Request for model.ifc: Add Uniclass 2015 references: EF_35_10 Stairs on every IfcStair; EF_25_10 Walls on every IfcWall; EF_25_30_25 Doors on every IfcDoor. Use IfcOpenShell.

First a look at what the model holds.

```python
import ifcopenshell

model = ifcopenshell.open("model.ifc")
print(model.schema)
print("classifications:", [c.Name for c in model.by_type("IfcClassification")])
for ifc_class in ("IfcDoor", "IfcRoof", "IfcStair", "IfcWall", "IfcWindow"):
    print(ifc_class, len(model.by_type(ifc_class)))
```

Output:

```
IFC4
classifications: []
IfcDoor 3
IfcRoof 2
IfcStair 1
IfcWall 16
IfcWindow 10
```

```python
import ifcopenshell
import ifcopenshell.api.classification

model = ifcopenshell.open("model.ifc")

system = ifcopenshell.api.classification.add_classification(model, classification="Uniclass 2015")

codes = {
    "IfcStair": ("EF_35_10", "Stairs"),
    "IfcWall": ("EF_25_10", "Walls"),
    "IfcDoor": ("EF_25_30_25", "Doors"),
}
for ifc_class, (code, name) in codes.items():
    products = model.by_type(ifc_class)
    ifcopenshell.api.classification.add_reference(
        model, products=products, classification=system, identification=code, name=name
    )
    print(code, len(products))

model.write("model_edited.ifc")
```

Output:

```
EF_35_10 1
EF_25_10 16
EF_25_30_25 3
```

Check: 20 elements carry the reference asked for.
